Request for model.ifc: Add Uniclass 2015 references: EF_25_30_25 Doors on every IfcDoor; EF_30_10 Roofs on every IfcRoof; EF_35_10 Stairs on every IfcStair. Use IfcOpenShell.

First a look at what the model holds.

```python
import ifcopenshell

model = ifcopenshell.open("model.ifc")
print(model.schema)
print("classifications:", [c.Name for c in model.by_type("IfcClassification")])
for ifc_class in ("IfcDoor", "IfcRoof", "IfcStair", "IfcWall", "IfcWindow"):
    print(ifc_class, len(model.by_type(ifc_class)))
```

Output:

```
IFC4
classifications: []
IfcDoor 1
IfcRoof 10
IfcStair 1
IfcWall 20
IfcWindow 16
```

```python
import ifcopenshell
import ifcopenshell.api.classification

model = ifcopenshell.open("model.ifc")

system = ifcopenshell.api.classification.add_classification(model, classification="Uniclass 2015")

codes = {
    "IfcDoor": ("EF_25_30_25", "Doors"),
    "IfcRoof": ("EF_30_10", "Roofs"),
    "IfcStair": ("EF_35_10", "Stairs"),
}
for ifc_class, (code, name) in codes.items():
    products = model.by_type(ifc_class)
    ifcopenshell.api.classification.add_reference(
        model, products=products, classification=system, identification=code, name=name
    )
    print(code, len(products))

model.write("model-out.ifc")
```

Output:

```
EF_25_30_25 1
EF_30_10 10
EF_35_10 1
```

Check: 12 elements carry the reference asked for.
